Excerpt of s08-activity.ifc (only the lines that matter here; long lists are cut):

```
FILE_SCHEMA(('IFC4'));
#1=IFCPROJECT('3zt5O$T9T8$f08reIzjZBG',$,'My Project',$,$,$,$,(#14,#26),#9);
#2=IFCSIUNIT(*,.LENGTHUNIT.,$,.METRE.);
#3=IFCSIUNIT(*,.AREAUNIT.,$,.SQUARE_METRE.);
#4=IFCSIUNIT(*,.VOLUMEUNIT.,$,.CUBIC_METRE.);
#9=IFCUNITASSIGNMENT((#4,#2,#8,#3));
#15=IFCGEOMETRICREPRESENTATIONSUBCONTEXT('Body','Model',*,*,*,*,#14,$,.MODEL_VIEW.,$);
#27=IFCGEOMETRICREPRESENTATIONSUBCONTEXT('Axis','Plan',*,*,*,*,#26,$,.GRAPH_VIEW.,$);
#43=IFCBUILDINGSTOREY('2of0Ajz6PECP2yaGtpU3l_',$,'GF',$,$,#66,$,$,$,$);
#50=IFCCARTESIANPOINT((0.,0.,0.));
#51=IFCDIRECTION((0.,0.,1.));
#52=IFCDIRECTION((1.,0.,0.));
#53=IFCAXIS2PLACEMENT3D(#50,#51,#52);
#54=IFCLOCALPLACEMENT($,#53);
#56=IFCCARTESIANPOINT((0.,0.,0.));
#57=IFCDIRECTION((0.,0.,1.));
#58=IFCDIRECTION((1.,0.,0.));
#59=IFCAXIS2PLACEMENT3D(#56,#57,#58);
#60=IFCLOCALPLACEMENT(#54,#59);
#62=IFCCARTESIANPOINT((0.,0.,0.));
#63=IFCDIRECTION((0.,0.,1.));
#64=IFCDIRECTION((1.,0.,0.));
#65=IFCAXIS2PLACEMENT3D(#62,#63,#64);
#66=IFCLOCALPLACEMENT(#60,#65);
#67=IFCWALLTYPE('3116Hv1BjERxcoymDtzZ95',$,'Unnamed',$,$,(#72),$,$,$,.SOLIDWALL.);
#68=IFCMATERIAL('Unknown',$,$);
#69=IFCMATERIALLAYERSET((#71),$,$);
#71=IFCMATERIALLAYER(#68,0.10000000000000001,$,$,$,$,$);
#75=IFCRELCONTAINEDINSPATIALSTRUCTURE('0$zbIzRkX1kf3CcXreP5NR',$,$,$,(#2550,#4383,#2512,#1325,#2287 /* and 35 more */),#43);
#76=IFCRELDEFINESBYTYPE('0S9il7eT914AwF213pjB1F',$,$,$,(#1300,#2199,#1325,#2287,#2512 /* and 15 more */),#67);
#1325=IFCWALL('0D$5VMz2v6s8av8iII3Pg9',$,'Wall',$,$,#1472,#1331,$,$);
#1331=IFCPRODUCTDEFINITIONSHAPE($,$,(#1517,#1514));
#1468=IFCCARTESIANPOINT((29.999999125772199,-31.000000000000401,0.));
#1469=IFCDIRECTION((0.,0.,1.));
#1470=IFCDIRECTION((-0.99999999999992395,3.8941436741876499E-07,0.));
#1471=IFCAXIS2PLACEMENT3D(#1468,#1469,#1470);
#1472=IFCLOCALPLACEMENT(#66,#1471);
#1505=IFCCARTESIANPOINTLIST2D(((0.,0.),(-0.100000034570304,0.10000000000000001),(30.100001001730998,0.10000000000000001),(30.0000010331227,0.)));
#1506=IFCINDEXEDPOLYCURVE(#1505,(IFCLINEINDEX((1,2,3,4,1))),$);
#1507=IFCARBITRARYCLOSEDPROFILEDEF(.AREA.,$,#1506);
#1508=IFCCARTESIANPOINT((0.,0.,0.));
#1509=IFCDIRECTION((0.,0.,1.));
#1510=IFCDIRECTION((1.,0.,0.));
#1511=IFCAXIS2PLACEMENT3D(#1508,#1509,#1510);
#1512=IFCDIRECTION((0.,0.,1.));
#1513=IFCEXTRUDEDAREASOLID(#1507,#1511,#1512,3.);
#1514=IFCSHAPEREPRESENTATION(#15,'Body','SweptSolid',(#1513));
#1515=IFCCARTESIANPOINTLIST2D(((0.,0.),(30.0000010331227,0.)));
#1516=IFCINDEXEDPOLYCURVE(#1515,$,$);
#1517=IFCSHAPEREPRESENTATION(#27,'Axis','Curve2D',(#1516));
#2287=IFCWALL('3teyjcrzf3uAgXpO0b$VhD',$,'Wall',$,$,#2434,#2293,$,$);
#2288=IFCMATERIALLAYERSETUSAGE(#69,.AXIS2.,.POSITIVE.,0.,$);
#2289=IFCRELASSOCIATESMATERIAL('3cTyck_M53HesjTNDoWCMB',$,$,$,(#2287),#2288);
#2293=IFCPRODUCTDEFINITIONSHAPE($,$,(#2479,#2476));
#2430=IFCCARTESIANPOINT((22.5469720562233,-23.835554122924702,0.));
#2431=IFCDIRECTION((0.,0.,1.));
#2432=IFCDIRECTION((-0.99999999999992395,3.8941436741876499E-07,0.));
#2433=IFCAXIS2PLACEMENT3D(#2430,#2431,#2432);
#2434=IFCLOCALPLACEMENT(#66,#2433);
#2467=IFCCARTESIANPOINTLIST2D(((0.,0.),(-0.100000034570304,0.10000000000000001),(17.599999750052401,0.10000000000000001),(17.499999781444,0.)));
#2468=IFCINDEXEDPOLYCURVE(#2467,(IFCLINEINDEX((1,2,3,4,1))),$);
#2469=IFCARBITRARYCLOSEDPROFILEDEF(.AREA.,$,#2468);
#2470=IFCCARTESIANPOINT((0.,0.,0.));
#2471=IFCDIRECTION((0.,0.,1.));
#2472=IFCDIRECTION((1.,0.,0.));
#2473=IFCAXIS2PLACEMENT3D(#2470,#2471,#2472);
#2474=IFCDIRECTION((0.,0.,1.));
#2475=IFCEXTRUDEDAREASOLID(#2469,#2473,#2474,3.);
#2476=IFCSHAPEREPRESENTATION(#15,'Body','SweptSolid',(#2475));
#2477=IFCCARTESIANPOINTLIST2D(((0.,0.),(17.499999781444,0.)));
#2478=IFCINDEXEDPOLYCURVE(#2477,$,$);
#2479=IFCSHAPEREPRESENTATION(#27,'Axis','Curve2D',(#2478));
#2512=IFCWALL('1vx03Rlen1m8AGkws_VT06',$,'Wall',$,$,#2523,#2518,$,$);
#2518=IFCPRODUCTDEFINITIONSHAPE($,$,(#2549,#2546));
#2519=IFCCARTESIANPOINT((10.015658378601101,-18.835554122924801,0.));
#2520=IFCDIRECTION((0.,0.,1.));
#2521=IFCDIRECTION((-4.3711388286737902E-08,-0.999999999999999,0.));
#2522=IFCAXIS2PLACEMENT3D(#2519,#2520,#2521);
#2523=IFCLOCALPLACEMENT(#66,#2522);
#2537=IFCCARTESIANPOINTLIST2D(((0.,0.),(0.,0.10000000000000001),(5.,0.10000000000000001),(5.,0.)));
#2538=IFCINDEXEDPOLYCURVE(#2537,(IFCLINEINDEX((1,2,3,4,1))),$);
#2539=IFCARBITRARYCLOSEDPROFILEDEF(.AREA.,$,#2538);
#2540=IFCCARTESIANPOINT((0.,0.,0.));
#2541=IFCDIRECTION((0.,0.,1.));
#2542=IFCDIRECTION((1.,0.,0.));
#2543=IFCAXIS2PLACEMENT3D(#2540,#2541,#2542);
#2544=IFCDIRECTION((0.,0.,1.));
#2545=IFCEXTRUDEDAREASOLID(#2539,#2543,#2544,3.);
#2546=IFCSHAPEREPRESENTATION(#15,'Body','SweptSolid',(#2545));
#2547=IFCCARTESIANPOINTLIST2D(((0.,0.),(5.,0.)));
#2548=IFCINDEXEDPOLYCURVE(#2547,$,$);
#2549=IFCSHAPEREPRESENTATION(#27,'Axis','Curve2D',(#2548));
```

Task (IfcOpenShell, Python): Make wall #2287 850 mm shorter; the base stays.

```python
import ifcopenshell
import ifcopenshell.geom
import ifcopenshell.util.representation
import ifcopenshell.util.shape

model = ifcopenshell.open("s08-activity.ifc")
settings = ifcopenshell.geom.settings()


def volume(element):
    """Net volume in cubic metres, openings subtracted."""
    shape = ifcopenshell.geom.create_shape(settings, element)
    return ifcopenshell.util.shape.get_volume(shape.geometry)


wall = model.by_guid("3teyjcrzf3uAgXpO0b$VhD")
before = volume(wall)

body = ifcopenshell.util.representation.get_representation(wall, "Model", "Body")
solid = body.Items[0]
old_height = solid.Depth
solid.Depth -= 0.85
after = volume(wall)

print(f"height {old_height:g} -> {solid.Depth:g}, volume {before:.3f} -> {after:.3f} m3")

model.write("s08-activity_rev.ifc")
```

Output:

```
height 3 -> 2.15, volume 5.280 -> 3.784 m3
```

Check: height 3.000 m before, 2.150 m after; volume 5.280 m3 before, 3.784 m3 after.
